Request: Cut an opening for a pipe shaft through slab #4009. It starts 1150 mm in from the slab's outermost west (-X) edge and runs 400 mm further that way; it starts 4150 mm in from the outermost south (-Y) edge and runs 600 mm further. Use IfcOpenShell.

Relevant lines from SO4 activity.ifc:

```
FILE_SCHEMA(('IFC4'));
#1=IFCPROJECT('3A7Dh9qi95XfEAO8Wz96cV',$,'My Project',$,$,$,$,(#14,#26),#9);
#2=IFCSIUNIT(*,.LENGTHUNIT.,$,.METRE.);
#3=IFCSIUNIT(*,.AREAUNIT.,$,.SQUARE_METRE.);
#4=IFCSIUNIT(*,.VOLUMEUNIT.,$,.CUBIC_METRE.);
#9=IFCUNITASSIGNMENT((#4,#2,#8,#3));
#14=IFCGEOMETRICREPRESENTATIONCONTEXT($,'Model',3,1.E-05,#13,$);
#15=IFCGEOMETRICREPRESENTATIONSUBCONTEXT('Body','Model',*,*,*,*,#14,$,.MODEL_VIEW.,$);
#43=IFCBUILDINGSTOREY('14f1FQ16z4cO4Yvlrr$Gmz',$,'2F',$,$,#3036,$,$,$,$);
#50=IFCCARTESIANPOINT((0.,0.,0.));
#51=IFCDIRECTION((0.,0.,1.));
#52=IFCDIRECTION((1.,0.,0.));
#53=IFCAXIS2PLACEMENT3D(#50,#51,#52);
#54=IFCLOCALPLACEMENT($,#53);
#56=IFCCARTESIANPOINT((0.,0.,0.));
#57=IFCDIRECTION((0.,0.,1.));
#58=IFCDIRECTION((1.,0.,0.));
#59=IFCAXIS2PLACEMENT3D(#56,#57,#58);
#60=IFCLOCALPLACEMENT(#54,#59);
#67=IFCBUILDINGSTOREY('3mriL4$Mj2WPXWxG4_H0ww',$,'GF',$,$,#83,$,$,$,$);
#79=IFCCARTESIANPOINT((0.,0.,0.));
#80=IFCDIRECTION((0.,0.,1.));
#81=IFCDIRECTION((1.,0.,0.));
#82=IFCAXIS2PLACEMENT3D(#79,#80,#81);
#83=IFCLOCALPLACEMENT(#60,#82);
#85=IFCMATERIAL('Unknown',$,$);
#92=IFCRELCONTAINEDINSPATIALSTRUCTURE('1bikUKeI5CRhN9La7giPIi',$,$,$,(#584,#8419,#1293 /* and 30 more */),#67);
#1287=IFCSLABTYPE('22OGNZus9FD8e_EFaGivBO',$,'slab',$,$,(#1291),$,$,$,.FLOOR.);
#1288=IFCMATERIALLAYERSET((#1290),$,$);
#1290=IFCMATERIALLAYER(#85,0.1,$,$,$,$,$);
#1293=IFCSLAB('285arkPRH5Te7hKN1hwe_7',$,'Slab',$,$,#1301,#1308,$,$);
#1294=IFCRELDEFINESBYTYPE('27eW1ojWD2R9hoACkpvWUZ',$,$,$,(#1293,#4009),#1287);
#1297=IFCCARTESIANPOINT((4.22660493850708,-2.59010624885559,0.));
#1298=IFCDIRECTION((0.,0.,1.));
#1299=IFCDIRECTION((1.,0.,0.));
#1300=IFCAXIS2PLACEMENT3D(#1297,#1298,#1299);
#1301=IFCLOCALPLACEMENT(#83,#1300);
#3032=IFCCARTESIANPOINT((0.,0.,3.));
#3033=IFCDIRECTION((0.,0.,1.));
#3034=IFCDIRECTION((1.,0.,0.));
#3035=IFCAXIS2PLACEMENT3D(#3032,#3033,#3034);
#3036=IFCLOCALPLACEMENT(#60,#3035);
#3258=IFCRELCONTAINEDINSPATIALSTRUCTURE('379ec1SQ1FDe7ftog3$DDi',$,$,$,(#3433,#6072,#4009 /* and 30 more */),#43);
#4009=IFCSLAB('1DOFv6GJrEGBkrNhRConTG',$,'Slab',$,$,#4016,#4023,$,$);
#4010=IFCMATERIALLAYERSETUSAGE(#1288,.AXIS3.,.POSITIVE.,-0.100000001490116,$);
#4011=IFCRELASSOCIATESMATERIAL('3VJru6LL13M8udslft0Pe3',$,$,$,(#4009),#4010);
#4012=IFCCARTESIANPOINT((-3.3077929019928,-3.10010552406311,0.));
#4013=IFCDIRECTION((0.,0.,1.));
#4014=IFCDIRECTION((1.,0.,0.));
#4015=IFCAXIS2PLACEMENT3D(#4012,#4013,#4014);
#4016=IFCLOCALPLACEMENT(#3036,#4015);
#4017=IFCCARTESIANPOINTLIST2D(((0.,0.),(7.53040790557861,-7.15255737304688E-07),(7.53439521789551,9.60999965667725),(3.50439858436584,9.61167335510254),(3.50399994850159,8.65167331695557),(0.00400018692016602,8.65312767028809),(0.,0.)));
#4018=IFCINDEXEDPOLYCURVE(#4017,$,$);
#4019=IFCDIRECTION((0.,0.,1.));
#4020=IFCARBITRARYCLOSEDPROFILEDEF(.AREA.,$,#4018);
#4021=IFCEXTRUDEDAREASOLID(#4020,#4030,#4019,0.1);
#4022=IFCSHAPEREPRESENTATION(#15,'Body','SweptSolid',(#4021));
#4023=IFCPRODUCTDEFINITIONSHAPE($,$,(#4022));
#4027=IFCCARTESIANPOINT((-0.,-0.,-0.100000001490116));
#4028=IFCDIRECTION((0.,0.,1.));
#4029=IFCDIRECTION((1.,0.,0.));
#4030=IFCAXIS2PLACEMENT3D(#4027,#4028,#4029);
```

```python
import numpy as np
import ifcopenshell
import ifcopenshell.api.feature
import ifcopenshell.api.geometry
import ifcopenshell.api.root
import ifcopenshell.geom
import ifcopenshell.util.placement
import ifcopenshell.util.representation
import ifcopenshell.util.shape
import ifcopenshell.util.unit

model = ifcopenshell.open("SO4 activity.ifc")
unit_scale = ifcopenshell.util.unit.calculate_unit_scale(model)
settings = ifcopenshell.geom.settings()


def volume(element):
    """Net volume in cubic metres, openings subtracted."""
    shape = ifcopenshell.geom.create_shape(settings, element)
    return ifcopenshell.util.shape.get_volume(shape.geometry)


slab = model.by_guid("1DOFv6GJrEGBkrNhRConTG")
before = volume(slab)

# Extent in the slab's own axes, in metres. The edges named are its -X and -Y sides.
slab_shape = ifcopenshell.geom.create_shape(settings, slab)
vertices = ifcopenshell.util.shape.get_vertices(slab_shape.geometry)
x_min, y_min, bottom = vertices.min(axis=0)
top = vertices[:, 2].max()

opening = ifcopenshell.api.root.create_entity(model, ifc_class="IfcOpeningElement", name="Pipe shaft opening", predefined_type="OPENING")
context = ifcopenshell.util.representation.get_context(model, "Model", "Body", "MODEL_VIEW")
width, depth = 0.4, 0.6
outline = [(0.0, 0.0), (width, 0.0), (width, depth), (0.0, depth), (0.0, 0.0)]
# Overshoot both faces by 50 mm so the cut is clean.
shape = ifcopenshell.api.geometry.add_slab_representation(
    model, context=context, depth=top - bottom + 0.1, polyline=outline
)
ifcopenshell.api.geometry.assign_representation(model, product=opening, representation=shape)

matrix = ifcopenshell.util.placement.get_local_placement(slab.ObjectPlacement)
matrix[:, 3] = matrix @ np.append(np.array([x_min + 1.15, y_min + 4.15, bottom - 0.05]) / unit_scale, 1.0)
ifcopenshell.api.geometry.edit_object_placement(model, product=opening, matrix=matrix, is_si=False)
ifcopenshell.api.feature.add_feature(model, feature=opening, element=slab)

after = volume(slab)

print(f"slab volume {before:.3f} -> {after:.3f} m3")

model.write("SO4 activity-out.ifc")
```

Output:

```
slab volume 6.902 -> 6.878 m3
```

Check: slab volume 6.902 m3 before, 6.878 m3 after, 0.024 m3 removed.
